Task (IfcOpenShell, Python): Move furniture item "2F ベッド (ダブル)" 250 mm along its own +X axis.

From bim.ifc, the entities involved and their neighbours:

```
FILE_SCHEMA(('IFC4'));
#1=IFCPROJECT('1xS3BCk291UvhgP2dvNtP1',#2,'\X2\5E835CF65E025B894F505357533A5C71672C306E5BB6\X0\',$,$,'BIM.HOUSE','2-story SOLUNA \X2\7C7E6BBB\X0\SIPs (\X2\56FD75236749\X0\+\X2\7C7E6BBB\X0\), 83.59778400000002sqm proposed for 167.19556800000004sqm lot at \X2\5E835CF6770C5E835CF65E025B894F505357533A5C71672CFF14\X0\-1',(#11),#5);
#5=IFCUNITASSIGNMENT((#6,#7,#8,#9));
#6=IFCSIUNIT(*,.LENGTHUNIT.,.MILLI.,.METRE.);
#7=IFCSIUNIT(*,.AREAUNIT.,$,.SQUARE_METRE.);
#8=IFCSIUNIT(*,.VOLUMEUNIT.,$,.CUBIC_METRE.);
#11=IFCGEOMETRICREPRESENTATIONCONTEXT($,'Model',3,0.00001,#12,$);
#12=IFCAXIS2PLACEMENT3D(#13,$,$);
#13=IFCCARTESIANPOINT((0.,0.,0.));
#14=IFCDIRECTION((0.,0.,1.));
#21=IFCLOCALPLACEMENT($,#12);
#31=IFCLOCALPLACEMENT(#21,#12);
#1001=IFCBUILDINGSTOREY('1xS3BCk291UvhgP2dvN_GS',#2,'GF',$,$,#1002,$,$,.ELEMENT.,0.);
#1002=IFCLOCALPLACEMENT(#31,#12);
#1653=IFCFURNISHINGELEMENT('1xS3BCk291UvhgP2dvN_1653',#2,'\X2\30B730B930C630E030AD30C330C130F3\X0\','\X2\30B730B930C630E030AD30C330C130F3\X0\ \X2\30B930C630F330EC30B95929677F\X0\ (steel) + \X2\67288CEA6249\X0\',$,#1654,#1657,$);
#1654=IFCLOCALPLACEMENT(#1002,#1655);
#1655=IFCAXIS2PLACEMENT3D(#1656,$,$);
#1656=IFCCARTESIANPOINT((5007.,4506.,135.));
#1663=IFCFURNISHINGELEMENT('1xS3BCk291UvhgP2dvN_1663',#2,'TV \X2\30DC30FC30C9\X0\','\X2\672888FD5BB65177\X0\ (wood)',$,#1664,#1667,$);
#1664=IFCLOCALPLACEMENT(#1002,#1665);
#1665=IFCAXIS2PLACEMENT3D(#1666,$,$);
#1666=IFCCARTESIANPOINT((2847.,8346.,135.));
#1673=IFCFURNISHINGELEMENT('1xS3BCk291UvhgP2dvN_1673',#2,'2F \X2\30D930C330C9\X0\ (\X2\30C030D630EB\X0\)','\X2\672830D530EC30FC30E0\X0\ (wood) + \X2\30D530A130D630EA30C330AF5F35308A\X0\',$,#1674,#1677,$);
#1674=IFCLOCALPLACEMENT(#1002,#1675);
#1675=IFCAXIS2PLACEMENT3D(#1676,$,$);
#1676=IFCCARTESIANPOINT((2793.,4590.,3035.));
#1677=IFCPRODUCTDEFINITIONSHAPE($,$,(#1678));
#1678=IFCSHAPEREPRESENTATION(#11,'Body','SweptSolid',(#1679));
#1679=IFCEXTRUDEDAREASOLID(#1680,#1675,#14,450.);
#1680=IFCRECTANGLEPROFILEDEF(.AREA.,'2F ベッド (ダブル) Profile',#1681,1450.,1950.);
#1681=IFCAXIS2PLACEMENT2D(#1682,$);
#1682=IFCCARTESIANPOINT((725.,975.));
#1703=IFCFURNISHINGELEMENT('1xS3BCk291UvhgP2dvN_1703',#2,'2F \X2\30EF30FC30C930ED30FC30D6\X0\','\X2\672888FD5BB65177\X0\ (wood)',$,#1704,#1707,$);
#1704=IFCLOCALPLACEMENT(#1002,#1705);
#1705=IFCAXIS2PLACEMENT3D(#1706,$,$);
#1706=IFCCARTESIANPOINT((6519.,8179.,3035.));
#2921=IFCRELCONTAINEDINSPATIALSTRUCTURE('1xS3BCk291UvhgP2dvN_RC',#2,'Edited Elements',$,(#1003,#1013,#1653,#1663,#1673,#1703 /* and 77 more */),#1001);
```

```python
import ifcopenshell
import ifcopenshell.api.geometry
import ifcopenshell.util.placement
import ifcopenshell.util.unit

model = ifcopenshell.open("bim.ifc")
unit_scale = ifcopenshell.util.unit.calculate_unit_scale(model)

item = model.by_id(1673)
matrix = ifcopenshell.util.placement.get_local_placement(item.ObjectPlacement)
matrix[:3, 3] += matrix[:3, 0] * 0.25 / unit_scale
ifcopenshell.api.geometry.edit_object_placement(model, product=item, matrix=matrix, is_si=False)

print(ifcopenshell.util.placement.get_local_placement(item.ObjectPlacement).round(3) + 0.0)

model.write("bim_rev.ifc")
```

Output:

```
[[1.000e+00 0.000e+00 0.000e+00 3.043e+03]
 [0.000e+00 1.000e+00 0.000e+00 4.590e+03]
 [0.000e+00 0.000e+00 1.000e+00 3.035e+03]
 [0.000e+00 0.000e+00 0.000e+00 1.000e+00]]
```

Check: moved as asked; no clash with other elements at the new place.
